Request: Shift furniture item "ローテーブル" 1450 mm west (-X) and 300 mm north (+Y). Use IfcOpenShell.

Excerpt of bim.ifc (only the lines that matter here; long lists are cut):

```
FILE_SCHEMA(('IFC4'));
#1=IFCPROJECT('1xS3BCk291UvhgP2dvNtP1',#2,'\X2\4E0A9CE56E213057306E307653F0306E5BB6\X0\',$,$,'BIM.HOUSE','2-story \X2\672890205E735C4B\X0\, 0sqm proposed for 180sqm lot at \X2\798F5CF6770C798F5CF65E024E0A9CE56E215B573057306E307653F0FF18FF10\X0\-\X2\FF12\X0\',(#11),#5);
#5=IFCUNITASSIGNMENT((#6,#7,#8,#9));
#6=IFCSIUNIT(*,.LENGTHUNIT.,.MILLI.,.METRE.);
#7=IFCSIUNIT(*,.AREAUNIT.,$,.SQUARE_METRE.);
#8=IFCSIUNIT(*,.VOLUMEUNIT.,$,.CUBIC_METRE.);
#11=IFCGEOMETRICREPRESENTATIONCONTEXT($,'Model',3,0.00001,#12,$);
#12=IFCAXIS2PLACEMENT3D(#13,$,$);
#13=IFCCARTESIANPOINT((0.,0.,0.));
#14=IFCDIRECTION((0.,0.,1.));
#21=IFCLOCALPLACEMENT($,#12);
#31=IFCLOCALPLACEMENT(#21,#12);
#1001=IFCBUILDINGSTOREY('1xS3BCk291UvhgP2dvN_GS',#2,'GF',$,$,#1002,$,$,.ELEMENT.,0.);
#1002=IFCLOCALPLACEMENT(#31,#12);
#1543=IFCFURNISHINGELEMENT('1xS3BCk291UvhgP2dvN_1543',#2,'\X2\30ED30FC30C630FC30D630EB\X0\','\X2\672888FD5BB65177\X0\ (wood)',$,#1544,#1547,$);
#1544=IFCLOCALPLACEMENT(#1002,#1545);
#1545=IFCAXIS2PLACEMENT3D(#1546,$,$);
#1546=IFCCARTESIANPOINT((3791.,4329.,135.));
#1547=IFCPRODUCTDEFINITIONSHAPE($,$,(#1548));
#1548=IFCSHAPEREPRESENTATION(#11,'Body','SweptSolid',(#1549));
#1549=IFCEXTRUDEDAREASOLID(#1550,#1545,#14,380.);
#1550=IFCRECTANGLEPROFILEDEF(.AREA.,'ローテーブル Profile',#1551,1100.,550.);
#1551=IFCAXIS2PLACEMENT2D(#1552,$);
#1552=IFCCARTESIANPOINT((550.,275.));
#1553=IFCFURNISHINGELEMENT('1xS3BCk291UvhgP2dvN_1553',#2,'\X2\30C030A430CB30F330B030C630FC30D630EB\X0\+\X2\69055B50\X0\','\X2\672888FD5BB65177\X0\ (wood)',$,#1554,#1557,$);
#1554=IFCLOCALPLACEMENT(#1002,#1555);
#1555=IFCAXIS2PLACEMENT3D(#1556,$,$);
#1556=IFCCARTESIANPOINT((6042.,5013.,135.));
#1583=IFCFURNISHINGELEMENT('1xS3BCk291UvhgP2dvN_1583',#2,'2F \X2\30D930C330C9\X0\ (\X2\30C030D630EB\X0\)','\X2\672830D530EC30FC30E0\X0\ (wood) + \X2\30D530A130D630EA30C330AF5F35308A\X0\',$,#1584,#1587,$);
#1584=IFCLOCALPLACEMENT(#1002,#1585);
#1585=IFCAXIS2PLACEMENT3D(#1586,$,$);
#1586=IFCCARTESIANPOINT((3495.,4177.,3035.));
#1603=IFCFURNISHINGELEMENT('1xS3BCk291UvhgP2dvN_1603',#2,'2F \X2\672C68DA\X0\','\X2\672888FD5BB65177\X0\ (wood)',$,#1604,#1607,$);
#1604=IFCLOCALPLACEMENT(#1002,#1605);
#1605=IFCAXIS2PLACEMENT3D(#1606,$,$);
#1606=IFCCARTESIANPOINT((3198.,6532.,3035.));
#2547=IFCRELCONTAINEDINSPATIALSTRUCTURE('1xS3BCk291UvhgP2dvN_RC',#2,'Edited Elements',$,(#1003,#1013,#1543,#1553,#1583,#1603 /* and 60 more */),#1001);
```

```python
import ifcopenshell
import ifcopenshell.api.geometry
import ifcopenshell.util.placement
import ifcopenshell.util.unit

model = ifcopenshell.open("bim.ifc")
unit_scale = ifcopenshell.util.unit.calculate_unit_scale(model)

item = model.by_id(1543)
matrix = ifcopenshell.util.placement.get_local_placement(item.ObjectPlacement)
matrix[0, 3] -= 1.45 / unit_scale
matrix[1, 3] += 0.3 / unit_scale
ifcopenshell.api.geometry.edit_object_placement(model, product=item, matrix=matrix, is_si=False)

print(ifcopenshell.util.placement.get_local_placement(item.ObjectPlacement).round(3) + 0.0)

model.write("bim_rev.ifc")
```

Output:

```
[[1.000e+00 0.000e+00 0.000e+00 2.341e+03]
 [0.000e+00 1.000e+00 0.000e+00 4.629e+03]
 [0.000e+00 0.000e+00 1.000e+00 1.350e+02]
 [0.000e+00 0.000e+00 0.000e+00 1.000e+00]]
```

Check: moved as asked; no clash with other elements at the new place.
